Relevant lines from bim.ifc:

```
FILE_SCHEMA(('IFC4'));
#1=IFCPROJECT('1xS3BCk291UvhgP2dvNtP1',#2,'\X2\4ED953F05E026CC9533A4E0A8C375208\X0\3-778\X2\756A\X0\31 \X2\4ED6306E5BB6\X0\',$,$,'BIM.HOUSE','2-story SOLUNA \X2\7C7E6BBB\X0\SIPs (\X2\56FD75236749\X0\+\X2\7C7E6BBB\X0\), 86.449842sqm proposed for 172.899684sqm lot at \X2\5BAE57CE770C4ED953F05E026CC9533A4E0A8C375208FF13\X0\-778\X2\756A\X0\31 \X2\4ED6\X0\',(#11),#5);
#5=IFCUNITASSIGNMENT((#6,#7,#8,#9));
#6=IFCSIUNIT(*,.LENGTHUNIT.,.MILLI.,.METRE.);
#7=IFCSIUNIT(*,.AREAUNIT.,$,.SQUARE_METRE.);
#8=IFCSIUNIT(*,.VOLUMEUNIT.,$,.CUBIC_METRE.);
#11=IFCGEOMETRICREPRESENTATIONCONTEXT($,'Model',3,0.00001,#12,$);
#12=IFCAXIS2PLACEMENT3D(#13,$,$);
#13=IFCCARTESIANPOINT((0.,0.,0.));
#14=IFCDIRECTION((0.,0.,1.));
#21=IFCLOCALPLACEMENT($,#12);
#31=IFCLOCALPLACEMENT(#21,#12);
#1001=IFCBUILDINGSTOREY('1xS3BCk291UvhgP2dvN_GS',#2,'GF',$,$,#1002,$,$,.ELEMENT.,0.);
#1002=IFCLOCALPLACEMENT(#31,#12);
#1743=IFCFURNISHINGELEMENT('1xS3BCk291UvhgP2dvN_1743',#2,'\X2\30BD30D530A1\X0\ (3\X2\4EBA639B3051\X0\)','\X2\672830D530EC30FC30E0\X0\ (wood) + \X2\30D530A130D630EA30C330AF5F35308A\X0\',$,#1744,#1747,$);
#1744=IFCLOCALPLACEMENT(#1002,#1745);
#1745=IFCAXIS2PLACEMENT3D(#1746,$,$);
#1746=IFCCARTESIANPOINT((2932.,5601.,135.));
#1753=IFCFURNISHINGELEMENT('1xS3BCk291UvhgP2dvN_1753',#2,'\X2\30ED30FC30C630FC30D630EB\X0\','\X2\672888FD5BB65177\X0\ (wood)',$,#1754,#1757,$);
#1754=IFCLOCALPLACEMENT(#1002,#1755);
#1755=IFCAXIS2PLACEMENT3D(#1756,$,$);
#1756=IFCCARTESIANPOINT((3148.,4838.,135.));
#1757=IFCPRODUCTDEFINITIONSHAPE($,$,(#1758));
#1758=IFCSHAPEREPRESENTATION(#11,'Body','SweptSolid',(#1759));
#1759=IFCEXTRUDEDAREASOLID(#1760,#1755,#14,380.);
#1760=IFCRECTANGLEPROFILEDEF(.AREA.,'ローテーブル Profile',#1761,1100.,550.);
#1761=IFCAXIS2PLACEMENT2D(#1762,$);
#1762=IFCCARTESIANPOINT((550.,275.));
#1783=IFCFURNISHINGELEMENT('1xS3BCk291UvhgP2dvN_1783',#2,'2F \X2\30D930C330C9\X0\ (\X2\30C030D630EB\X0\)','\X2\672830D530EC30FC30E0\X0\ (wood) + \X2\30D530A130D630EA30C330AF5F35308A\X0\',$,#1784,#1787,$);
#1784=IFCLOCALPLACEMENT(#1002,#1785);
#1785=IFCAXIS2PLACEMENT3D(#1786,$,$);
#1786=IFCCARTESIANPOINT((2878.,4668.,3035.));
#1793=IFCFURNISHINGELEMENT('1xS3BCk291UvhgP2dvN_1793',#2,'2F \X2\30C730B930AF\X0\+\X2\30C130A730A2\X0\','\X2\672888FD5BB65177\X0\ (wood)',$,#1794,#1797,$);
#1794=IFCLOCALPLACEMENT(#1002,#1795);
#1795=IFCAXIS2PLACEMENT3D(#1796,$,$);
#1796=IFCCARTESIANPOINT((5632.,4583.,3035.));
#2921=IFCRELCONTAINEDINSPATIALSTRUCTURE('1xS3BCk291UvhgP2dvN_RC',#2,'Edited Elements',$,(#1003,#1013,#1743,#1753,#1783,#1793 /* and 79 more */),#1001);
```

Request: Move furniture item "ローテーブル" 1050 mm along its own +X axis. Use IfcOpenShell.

```python
import ifcopenshell
import ifcopenshell.api.geometry
import ifcopenshell.util.placement
import ifcopenshell.util.unit

model = ifcopenshell.open("bim.ifc")
unit_scale = ifcopenshell.util.unit.calculate_unit_scale(model)

item = model.by_id(1753)
matrix = ifcopenshell.util.placement.get_local_placement(item.ObjectPlacement)
matrix[:3, 3] += matrix[:3, 0] * 1.05 / unit_scale
ifcopenshell.api.geometry.edit_object_placement(model, product=item, matrix=matrix, is_si=False)

print(ifcopenshell.util.placement.get_local_placement(item.ObjectPlacement).round(3) + 0.0)

model.write("bim_updated.ifc")
```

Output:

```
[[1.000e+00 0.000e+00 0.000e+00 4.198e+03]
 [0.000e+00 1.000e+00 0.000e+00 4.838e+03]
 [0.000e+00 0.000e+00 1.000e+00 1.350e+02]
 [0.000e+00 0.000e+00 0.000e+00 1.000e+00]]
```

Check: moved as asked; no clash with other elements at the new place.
